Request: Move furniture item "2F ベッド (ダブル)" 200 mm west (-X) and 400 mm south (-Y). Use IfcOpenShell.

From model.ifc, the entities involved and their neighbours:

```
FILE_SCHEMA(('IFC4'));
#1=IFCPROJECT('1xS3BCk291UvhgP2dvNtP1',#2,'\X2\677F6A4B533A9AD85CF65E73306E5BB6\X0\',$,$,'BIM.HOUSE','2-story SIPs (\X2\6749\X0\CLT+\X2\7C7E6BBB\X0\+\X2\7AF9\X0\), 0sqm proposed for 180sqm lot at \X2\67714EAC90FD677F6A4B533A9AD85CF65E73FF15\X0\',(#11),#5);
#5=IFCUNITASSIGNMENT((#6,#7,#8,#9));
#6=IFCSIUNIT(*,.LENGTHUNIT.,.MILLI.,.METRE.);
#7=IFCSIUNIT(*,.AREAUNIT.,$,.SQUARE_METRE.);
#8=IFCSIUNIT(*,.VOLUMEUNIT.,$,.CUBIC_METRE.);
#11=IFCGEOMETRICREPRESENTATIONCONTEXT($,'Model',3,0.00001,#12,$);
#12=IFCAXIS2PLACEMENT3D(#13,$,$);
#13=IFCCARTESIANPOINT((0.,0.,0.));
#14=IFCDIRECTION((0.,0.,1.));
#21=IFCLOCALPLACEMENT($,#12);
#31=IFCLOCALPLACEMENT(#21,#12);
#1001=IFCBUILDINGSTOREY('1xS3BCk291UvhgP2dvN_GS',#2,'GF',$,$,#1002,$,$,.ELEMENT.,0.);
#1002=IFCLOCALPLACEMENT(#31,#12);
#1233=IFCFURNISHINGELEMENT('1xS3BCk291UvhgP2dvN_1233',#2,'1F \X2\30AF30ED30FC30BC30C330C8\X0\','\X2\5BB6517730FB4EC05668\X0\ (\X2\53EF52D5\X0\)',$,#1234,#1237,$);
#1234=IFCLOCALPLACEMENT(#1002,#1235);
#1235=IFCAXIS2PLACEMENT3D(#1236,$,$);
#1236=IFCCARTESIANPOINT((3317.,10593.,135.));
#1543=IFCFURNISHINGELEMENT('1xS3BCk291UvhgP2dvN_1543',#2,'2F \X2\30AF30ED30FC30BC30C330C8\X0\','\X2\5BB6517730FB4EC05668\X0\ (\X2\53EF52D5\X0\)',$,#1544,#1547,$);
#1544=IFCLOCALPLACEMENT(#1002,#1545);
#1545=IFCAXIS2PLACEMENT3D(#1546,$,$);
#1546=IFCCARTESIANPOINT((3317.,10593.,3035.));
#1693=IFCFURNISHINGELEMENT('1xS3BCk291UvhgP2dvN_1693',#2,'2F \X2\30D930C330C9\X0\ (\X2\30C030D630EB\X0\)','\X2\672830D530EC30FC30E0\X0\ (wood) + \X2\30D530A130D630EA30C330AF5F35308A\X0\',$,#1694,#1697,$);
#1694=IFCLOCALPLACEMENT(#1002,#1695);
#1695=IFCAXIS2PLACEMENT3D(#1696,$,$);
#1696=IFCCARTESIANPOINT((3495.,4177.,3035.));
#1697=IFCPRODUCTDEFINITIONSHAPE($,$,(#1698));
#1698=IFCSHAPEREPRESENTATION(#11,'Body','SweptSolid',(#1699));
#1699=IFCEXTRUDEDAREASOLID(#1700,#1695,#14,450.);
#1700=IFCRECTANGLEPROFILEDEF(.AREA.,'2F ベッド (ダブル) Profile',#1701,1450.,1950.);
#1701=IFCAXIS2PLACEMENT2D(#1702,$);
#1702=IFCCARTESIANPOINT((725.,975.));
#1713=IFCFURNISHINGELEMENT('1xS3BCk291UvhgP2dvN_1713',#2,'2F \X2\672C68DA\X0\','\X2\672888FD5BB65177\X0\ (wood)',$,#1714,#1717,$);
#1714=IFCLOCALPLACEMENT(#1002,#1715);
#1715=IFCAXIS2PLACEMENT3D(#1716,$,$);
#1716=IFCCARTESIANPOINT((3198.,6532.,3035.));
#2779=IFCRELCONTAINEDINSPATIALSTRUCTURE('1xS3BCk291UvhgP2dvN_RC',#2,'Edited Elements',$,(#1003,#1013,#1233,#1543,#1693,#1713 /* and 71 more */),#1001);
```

```python
import ifcopenshell
import ifcopenshell.api.geometry
import ifcopenshell.util.placement
import ifcopenshell.util.unit

model = ifcopenshell.open("model.ifc")
unit_scale = ifcopenshell.util.unit.calculate_unit_scale(model)

item = model.by_guid("1xS3BCk291UvhgP2dvN_1693")
matrix = ifcopenshell.util.placement.get_local_placement(item.ObjectPlacement)
matrix[0, 3] -= 0.2 / unit_scale
matrix[1, 3] -= 0.4 / unit_scale
ifcopenshell.api.geometry.edit_object_placement(model, product=item, matrix=matrix, is_si=False)

print(ifcopenshell.util.placement.get_local_placement(item.ObjectPlacement).round(3) + 0.0)

model.write("model_updated.ifc")
```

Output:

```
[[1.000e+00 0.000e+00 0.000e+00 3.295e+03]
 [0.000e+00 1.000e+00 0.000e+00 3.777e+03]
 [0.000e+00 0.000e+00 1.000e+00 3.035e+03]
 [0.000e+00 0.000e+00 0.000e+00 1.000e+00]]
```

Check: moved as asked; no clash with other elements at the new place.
